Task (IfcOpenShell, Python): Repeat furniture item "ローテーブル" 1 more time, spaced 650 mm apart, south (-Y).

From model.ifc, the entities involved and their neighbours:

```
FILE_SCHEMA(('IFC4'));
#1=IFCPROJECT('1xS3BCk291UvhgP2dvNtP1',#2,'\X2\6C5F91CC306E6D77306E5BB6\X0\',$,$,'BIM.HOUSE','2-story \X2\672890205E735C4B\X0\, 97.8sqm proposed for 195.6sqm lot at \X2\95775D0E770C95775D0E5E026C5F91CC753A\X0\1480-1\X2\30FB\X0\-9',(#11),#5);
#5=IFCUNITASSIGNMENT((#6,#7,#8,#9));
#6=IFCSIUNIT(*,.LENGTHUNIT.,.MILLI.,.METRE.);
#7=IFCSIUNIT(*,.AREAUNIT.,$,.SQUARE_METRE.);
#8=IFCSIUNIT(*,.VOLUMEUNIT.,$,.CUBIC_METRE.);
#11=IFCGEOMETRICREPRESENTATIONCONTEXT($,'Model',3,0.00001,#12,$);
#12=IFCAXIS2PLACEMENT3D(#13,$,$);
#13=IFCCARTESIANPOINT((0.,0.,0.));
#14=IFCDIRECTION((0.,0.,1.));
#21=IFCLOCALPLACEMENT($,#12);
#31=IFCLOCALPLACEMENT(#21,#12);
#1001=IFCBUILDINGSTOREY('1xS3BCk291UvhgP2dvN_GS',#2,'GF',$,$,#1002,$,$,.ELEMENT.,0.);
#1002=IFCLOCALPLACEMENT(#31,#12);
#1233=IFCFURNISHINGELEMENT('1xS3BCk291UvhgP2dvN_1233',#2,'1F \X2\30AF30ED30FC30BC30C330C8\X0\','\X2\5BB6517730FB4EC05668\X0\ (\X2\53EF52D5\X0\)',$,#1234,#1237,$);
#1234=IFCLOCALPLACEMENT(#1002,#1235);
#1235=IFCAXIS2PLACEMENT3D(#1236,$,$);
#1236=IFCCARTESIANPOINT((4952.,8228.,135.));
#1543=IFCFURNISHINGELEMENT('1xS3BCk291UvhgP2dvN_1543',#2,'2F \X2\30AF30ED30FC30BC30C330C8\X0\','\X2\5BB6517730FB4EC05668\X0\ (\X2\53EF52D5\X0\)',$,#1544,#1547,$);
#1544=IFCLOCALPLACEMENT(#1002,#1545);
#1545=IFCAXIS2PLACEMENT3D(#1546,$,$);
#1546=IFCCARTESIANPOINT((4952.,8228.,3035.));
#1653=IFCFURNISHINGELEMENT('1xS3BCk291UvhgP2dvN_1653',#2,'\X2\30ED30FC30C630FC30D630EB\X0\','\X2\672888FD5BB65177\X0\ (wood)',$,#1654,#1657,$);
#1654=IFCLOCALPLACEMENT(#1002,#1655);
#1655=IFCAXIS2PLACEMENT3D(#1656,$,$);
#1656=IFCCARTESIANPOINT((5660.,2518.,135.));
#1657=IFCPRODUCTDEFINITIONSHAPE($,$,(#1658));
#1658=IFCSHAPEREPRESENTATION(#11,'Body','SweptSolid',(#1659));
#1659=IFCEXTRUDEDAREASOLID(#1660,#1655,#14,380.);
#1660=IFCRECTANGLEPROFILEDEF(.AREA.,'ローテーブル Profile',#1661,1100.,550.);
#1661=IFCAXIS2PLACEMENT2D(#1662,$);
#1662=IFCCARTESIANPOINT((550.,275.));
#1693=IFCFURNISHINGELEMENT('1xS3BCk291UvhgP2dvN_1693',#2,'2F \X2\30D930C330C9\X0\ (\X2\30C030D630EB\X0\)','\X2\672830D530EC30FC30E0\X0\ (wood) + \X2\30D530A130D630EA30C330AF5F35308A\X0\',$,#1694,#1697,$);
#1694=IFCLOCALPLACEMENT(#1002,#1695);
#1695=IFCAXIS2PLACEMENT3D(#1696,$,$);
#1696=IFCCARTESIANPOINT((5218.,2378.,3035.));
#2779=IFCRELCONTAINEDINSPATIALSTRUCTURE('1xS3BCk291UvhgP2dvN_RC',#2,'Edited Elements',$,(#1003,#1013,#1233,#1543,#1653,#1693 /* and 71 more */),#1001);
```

```python
import numpy as np
import ifcopenshell
import ifcopenshell.api.geometry
import ifcopenshell.api.root
import ifcopenshell.util.element
import ifcopenshell.util.placement
import ifcopenshell.util.unit

model = ifcopenshell.open("model.ifc")
unit_scale = ifcopenshell.util.unit.calculate_unit_scale(model)


def reuse_history(source, copy):
    """copy_class also copies each property set's owner history, people and application; keep the originals."""
    for rel in copy.IsDefinedBy:
        if rel.is_a("IfcRelDefinesByProperties") and (history := rel.RelatingPropertyDefinition.OwnerHistory):
            rel.RelatingPropertyDefinition.OwnerHistory = source.OwnerHistory
            ifcopenshell.util.element.remove_deep2(model, history)


source = model.by_guid("1xS3BCk291UvhgP2dvN_1653")
base = ifcopenshell.util.placement.get_local_placement(source.ObjectPlacement)
step = np.array([0.0, -1.0, 0.0]) * 0.65 / unit_scale

for i in range(1, 2):
    copy = ifcopenshell.api.root.copy_class(model, product=source)
    copy.Representation = ifcopenshell.util.element.copy_deep(
        model, source.Representation, exclude=["IfcGeometricRepresentationContext", "IfcRepresentationMap"]
    )
    reuse_history(source, copy)
    matrix = base.copy()
    matrix[:3, 3] += i * step
    print("added at", matrix[:3, 3].round(3) + 0.0)
    ifcopenshell.api.geometry.edit_object_placement(model, product=copy, matrix=matrix, is_si=False)

model.write("model-out.ifc")
```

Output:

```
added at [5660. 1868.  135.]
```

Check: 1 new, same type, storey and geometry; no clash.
